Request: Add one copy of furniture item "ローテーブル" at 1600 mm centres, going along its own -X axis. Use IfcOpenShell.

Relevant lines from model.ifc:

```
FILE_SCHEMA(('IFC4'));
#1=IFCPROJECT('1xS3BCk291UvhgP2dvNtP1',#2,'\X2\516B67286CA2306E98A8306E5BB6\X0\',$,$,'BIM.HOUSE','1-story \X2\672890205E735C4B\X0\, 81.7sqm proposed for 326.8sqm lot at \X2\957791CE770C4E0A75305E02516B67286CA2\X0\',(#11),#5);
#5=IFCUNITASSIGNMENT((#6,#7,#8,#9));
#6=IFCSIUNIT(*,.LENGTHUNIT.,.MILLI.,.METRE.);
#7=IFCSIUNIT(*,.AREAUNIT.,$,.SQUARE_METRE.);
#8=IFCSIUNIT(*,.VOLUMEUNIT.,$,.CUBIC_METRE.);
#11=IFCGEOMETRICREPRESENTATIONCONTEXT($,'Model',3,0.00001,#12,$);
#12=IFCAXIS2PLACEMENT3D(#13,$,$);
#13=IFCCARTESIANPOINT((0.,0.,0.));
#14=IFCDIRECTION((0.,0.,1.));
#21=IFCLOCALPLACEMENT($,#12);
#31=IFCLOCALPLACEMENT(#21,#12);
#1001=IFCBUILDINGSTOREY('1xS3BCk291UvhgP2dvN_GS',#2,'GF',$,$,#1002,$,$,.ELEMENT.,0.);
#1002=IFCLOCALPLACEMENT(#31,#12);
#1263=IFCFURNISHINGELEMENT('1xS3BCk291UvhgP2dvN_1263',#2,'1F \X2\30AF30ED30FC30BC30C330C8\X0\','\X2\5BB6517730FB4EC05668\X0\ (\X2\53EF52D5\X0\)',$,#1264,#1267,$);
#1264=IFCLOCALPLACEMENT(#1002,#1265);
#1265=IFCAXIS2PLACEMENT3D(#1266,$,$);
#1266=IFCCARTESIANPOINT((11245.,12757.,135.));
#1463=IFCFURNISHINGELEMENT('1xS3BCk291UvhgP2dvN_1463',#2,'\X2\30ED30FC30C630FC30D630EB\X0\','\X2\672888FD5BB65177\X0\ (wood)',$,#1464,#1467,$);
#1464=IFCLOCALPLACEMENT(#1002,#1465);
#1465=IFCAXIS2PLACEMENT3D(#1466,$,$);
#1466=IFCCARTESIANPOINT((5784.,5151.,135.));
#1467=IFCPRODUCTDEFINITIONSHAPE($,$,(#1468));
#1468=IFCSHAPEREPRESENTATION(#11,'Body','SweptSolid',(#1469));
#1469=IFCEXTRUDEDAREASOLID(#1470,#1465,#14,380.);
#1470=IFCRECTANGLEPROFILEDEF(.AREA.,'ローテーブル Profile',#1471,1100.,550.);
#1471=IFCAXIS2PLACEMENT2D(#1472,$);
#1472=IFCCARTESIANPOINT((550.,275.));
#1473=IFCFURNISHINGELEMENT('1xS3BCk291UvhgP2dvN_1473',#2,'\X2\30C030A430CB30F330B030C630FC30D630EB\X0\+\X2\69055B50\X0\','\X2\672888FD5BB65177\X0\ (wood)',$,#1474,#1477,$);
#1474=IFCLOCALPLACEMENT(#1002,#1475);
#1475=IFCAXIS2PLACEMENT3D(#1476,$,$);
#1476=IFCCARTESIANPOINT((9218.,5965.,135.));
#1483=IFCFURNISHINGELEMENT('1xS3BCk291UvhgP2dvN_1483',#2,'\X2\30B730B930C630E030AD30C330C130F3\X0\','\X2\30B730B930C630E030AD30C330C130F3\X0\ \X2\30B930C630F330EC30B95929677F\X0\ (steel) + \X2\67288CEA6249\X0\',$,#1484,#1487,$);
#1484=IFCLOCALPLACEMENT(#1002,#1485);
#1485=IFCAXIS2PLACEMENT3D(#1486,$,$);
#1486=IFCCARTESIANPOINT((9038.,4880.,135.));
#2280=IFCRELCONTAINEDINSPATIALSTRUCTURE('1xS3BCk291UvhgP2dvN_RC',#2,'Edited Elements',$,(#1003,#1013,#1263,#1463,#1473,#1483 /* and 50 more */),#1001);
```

```python
import ifcopenshell
import ifcopenshell.api.geometry
import ifcopenshell.api.root
import ifcopenshell.util.element
import ifcopenshell.util.placement
import ifcopenshell.util.unit

model = ifcopenshell.open("model.ifc")
unit_scale = ifcopenshell.util.unit.calculate_unit_scale(model)


def reuse_history(source, copy):
    """copy_class also copies each property set's owner history, people and application; keep the originals."""
    for rel in copy.IsDefinedBy:
        if rel.is_a("IfcRelDefinesByProperties") and (history := rel.RelatingPropertyDefinition.OwnerHistory):
            rel.RelatingPropertyDefinition.OwnerHistory = source.OwnerHistory
            ifcopenshell.util.element.remove_deep2(model, history)


source = model.by_id(1463)
base = ifcopenshell.util.placement.get_local_placement(source.ObjectPlacement)
step = -base[:3, 0] * 1.6 / unit_scale

for i in range(1, 2):
    copy = ifcopenshell.api.root.copy_class(model, product=source)
    copy.Representation = ifcopenshell.util.element.copy_deep(
        model, source.Representation, exclude=["IfcGeometricRepresentationContext", "IfcRepresentationMap"]
    )
    reuse_history(source, copy)
    matrix = base.copy()
    matrix[:3, 3] += i * step
    print("added at", matrix[:3, 3].round(3) + 0.0)
    ifcopenshell.api.geometry.edit_object_placement(model, product=copy, matrix=matrix, is_si=False)

model.write("model-out.ifc")
```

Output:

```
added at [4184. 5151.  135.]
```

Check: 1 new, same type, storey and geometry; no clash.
